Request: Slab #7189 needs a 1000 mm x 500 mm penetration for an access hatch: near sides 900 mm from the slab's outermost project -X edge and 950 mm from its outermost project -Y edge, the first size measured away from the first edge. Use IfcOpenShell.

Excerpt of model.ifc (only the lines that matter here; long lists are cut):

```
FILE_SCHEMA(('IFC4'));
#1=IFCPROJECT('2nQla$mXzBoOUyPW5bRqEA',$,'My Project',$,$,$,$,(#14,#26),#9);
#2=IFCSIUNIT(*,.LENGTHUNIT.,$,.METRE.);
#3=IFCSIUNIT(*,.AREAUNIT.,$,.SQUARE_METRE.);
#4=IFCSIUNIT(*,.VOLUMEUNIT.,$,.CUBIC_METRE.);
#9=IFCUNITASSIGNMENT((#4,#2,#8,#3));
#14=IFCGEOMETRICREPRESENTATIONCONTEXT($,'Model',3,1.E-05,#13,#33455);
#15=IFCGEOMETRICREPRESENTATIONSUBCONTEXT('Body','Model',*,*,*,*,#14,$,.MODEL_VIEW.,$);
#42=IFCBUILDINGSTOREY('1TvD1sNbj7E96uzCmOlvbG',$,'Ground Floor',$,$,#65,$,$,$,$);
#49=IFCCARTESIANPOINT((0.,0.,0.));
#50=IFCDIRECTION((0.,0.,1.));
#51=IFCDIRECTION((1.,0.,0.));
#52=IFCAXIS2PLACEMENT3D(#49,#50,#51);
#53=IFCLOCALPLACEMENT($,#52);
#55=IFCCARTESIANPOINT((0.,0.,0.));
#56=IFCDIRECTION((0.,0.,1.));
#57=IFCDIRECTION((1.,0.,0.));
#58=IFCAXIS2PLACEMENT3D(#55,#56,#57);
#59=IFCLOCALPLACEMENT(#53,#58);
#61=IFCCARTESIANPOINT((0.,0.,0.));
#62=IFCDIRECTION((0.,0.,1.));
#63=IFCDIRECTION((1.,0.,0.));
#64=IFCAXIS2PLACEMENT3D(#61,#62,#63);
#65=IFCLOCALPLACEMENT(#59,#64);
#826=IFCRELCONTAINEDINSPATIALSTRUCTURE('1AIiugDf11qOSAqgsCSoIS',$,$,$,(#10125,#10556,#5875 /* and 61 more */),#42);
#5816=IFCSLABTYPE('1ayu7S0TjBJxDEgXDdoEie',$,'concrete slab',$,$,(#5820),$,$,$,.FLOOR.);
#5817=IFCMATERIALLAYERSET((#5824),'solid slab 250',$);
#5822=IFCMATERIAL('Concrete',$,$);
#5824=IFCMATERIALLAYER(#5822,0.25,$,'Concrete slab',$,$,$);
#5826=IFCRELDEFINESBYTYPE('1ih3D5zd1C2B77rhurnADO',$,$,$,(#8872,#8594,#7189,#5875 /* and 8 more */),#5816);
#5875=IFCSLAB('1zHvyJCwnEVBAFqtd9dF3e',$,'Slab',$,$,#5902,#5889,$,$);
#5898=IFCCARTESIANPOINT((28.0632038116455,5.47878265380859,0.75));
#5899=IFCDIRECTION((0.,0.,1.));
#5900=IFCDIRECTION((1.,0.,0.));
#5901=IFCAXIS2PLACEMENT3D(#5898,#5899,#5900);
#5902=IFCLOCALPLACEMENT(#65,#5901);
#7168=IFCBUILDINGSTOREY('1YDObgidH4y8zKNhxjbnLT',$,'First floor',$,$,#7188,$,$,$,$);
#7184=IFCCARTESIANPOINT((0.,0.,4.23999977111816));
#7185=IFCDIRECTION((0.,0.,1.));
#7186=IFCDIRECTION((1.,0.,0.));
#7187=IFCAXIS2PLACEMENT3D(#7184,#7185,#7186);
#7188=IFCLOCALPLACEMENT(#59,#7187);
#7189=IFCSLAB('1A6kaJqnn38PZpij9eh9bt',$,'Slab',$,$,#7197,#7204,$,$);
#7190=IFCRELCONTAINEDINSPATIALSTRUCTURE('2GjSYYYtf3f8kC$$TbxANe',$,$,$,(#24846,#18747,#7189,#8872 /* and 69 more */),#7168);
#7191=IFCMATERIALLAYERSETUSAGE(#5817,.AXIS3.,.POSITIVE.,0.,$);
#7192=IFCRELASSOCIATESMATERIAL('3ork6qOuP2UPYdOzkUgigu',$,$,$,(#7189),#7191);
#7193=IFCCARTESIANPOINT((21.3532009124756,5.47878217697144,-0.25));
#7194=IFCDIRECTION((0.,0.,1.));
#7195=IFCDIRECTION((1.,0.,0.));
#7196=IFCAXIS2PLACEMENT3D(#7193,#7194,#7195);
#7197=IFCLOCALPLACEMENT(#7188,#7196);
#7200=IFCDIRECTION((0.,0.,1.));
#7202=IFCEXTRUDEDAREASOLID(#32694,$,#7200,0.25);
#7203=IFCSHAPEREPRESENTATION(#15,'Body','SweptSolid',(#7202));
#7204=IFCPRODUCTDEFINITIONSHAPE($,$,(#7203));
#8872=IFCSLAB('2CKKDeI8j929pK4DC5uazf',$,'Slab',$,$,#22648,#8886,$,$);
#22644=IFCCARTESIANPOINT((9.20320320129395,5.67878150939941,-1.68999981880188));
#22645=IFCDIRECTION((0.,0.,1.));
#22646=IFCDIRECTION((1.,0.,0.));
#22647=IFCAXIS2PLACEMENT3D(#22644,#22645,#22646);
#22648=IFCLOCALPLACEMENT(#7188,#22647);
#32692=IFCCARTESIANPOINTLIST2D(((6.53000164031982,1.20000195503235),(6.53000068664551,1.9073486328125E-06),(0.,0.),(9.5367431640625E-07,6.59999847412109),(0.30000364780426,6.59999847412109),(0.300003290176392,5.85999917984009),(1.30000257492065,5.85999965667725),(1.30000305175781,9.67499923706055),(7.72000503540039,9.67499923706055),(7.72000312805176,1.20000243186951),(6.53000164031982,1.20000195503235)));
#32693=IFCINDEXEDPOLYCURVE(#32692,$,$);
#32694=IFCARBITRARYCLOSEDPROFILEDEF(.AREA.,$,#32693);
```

```python
import numpy as np
import ifcopenshell
import ifcopenshell.api.feature
import ifcopenshell.api.geometry
import ifcopenshell.api.root
import ifcopenshell.geom
import ifcopenshell.util.placement
import ifcopenshell.util.representation
import ifcopenshell.util.shape
import ifcopenshell.util.unit

model = ifcopenshell.open("model.ifc")
unit_scale = ifcopenshell.util.unit.calculate_unit_scale(model)
settings = ifcopenshell.geom.settings()


def volume(element):
    """Net volume in cubic metres, openings subtracted."""
    shape = ifcopenshell.geom.create_shape(settings, element)
    return ifcopenshell.util.shape.get_volume(shape.geometry)


slab = model.by_guid("1A6kaJqnn38PZpij9eh9bt")
before = volume(slab)

# Extent in the slab's own axes, in metres. The edges named are its -X and -Y sides.
slab_shape = ifcopenshell.geom.create_shape(settings, slab)
vertices = ifcopenshell.util.shape.get_vertices(slab_shape.geometry)
x_min, y_min, bottom = vertices.min(axis=0)
top = vertices[:, 2].max()

opening = ifcopenshell.api.root.create_entity(model, ifc_class="IfcOpeningElement", name="Access hatch opening", predefined_type="OPENING")
context = ifcopenshell.util.representation.get_context(model, "Model", "Body", "MODEL_VIEW")
width, depth = 1, 0.5
outline = [(0.0, 0.0), (width, 0.0), (width, depth), (0.0, depth), (0.0, 0.0)]
# Overshoot both faces by 50 mm so the cut is clean.
shape = ifcopenshell.api.geometry.add_slab_representation(
    model, context=context, depth=top - bottom + 0.1, polyline=outline
)
ifcopenshell.api.geometry.assign_representation(model, product=opening, representation=shape)

matrix = ifcopenshell.util.placement.get_local_placement(slab.ObjectPlacement)
matrix[:, 3] = matrix @ np.append(np.array([x_min + 0.9, y_min + 0.95, bottom - 0.05]) / unit_scale, 1.0)
ifcopenshell.api.geometry.edit_object_placement(model, product=opening, matrix=matrix, is_si=False)
ifcopenshell.api.feature.add_feature(model, feature=opening, element=slab)

after = volume(slab)

print(f"slab volume {before:.3f} -> {after:.3f} m3")

model.write("model_rev.ifc")
```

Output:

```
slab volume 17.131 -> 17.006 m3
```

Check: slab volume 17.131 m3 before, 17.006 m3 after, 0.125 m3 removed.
